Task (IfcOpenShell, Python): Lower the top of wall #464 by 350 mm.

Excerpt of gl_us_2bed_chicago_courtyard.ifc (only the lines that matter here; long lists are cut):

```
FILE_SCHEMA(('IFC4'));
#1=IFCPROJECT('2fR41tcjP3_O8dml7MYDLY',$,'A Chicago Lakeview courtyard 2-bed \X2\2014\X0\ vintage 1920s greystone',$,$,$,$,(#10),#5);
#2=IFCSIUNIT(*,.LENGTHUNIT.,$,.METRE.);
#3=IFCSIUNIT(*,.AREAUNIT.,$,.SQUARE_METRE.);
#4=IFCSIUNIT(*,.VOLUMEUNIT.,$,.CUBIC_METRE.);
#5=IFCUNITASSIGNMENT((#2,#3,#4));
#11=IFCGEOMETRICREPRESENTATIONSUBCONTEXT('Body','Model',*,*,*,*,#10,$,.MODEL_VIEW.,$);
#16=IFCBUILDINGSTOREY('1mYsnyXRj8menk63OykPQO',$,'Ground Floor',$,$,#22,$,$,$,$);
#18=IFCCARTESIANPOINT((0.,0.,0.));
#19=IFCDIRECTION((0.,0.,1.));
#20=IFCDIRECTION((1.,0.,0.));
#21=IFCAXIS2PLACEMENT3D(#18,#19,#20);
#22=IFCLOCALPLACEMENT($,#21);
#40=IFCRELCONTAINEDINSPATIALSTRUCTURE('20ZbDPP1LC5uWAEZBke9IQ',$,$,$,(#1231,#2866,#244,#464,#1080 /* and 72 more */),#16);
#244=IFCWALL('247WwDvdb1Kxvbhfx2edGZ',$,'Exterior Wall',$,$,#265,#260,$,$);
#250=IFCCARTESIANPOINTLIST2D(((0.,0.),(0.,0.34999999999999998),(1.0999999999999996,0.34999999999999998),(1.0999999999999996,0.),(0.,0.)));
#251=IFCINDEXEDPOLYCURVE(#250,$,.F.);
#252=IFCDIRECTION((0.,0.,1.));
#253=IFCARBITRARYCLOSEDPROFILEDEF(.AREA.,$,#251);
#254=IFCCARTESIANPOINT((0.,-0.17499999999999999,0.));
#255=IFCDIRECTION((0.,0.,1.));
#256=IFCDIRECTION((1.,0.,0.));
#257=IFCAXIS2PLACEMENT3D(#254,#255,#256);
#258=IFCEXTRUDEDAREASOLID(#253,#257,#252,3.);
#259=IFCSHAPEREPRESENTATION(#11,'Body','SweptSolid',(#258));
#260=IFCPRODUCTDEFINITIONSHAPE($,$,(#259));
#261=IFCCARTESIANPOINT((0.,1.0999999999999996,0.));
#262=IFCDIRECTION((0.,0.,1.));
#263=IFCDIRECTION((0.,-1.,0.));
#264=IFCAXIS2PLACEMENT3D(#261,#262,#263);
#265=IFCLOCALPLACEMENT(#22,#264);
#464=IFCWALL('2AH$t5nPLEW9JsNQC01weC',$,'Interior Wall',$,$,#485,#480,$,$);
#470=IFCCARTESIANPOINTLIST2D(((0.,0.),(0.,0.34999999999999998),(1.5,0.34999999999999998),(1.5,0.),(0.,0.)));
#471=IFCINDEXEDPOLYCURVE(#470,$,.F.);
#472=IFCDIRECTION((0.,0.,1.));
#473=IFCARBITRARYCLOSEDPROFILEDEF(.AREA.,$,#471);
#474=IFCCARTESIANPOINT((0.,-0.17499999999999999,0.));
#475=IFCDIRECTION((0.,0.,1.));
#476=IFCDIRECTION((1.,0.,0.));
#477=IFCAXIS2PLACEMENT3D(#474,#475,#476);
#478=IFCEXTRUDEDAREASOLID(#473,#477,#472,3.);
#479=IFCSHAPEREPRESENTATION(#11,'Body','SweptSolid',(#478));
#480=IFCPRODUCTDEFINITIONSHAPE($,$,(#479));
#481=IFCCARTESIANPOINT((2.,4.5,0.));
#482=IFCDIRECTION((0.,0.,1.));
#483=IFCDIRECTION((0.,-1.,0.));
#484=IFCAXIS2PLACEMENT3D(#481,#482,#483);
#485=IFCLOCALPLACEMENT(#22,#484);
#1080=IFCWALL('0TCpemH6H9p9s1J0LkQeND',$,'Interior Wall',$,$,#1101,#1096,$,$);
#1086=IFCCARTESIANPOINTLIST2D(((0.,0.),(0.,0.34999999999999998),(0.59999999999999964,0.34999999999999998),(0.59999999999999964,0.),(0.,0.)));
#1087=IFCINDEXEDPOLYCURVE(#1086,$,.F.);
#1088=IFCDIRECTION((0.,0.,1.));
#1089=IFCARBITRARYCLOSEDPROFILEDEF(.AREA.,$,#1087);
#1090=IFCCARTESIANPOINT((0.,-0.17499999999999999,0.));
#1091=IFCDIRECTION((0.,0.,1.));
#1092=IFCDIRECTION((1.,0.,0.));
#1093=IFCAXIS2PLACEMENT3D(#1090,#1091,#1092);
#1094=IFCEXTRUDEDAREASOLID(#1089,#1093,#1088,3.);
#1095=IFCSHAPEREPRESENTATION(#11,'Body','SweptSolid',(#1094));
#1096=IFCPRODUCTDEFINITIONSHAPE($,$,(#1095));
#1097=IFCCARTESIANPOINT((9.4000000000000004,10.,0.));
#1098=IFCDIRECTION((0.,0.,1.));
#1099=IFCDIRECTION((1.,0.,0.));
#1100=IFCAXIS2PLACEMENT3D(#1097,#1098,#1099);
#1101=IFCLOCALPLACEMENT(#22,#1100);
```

```python
import ifcopenshell
import ifcopenshell.geom
import ifcopenshell.util.representation
import ifcopenshell.util.shape
import ifcopenshell.util.unit

model = ifcopenshell.open("gl_us_2bed_chicago_courtyard.ifc")
unit_scale = ifcopenshell.util.unit.calculate_unit_scale(model)
settings = ifcopenshell.geom.settings()


def volume(element):
    """Net volume in cubic metres, openings subtracted."""
    shape = ifcopenshell.geom.create_shape(settings, element)
    return ifcopenshell.util.shape.get_volume(shape.geometry)


wall = model.by_guid("2AH$t5nPLEW9JsNQC01weC")
before = volume(wall)

body = ifcopenshell.util.representation.get_representation(wall, "Model", "Body")
solid = body.Items[0]
old_height = solid.Depth
solid.Depth -= 0.35 / unit_scale
after = volume(wall)

print(f"height {old_height:g} -> {solid.Depth:g}, volume {before:.3f} -> {after:.3f} m3")

model.write("gl_us_2bed_chicago_courtyard_updated.ifc")
```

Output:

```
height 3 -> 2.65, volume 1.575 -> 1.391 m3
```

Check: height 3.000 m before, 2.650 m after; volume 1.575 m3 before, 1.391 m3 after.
